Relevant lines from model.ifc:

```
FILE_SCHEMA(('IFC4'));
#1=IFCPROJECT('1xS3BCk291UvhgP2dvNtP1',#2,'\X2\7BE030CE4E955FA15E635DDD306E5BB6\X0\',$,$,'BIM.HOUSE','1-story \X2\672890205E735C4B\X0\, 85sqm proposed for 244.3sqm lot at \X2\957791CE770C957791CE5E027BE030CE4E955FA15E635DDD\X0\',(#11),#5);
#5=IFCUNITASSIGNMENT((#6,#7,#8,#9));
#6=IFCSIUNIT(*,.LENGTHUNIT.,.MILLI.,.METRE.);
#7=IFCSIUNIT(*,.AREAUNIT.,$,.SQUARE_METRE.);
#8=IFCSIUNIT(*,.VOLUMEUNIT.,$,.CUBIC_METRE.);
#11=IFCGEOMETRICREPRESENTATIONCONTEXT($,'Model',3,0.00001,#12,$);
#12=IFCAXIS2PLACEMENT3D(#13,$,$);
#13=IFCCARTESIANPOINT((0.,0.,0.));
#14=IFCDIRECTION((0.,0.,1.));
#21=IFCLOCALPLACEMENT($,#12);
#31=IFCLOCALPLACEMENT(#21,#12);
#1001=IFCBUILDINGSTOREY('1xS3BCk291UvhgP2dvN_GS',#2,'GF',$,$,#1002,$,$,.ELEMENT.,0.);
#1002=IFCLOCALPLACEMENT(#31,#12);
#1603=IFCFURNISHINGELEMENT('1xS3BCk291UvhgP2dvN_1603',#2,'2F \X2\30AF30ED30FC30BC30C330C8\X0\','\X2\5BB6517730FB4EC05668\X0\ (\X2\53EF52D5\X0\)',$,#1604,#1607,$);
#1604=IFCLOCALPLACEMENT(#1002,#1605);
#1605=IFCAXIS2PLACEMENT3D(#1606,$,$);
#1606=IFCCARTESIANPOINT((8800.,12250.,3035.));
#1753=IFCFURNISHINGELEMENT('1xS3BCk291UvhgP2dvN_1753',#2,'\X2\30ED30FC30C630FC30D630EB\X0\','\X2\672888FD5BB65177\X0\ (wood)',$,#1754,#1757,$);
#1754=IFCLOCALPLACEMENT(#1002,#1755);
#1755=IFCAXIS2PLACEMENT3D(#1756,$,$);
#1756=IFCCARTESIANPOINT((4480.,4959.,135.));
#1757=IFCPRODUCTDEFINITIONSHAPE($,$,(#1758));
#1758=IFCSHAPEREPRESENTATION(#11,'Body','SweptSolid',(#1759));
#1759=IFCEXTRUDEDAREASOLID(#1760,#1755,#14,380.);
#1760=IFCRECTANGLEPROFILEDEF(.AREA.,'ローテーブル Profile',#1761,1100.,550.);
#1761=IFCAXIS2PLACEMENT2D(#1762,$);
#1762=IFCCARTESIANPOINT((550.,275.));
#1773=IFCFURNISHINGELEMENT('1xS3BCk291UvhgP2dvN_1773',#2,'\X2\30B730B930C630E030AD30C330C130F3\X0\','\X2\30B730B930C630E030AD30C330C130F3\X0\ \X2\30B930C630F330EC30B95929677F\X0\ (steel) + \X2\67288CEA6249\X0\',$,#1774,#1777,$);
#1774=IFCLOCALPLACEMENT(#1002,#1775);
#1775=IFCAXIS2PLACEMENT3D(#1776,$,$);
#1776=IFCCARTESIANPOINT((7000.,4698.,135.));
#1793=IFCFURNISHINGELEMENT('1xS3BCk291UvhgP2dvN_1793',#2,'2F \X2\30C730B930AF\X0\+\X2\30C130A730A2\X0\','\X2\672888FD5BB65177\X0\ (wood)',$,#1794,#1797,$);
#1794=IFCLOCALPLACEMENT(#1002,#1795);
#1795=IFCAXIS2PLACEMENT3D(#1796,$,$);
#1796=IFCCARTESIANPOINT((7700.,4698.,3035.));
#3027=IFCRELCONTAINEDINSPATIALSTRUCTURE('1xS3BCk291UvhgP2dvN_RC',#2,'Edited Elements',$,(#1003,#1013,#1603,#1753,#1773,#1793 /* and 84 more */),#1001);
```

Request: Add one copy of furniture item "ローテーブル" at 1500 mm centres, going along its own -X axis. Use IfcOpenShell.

```python
import ifcopenshell
import ifcopenshell.api.geometry
import ifcopenshell.api.root
import ifcopenshell.util.element
import ifcopenshell.util.placement
import ifcopenshell.util.unit

model = ifcopenshell.open("model.ifc")
unit_scale = ifcopenshell.util.unit.calculate_unit_scale(model)


def reuse_history(source, copy):
    """copy_class also copies each property set's owner history, people and application; keep the originals."""
    for rel in copy.IsDefinedBy:
        if rel.is_a("IfcRelDefinesByProperties") and (history := rel.RelatingPropertyDefinition.OwnerHistory):
            rel.RelatingPropertyDefinition.OwnerHistory = source.OwnerHistory
            ifcopenshell.util.element.remove_deep2(model, history)


source = model.by_guid("1xS3BCk291UvhgP2dvN_1753")
base = ifcopenshell.util.placement.get_local_placement(source.ObjectPlacement)
step = -base[:3, 0] * 1.5 / unit_scale

for i in range(1, 2):
    copy = ifcopenshell.api.root.copy_class(model, product=source)
    copy.Representation = ifcopenshell.util.element.copy_deep(
        model, source.Representation, exclude=["IfcGeometricRepresentationContext", "IfcRepresentationMap"]
    )
    reuse_history(source, copy)
    matrix = base.copy()
    matrix[:3, 3] += i * step
    print("added at", matrix[:3, 3].round(3) + 0.0)
    ifcopenshell.api.geometry.edit_object_placement(model, product=copy, matrix=matrix, is_si=False)

model.write("model_edited.ifc")
```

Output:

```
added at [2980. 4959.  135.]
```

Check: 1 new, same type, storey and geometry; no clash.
